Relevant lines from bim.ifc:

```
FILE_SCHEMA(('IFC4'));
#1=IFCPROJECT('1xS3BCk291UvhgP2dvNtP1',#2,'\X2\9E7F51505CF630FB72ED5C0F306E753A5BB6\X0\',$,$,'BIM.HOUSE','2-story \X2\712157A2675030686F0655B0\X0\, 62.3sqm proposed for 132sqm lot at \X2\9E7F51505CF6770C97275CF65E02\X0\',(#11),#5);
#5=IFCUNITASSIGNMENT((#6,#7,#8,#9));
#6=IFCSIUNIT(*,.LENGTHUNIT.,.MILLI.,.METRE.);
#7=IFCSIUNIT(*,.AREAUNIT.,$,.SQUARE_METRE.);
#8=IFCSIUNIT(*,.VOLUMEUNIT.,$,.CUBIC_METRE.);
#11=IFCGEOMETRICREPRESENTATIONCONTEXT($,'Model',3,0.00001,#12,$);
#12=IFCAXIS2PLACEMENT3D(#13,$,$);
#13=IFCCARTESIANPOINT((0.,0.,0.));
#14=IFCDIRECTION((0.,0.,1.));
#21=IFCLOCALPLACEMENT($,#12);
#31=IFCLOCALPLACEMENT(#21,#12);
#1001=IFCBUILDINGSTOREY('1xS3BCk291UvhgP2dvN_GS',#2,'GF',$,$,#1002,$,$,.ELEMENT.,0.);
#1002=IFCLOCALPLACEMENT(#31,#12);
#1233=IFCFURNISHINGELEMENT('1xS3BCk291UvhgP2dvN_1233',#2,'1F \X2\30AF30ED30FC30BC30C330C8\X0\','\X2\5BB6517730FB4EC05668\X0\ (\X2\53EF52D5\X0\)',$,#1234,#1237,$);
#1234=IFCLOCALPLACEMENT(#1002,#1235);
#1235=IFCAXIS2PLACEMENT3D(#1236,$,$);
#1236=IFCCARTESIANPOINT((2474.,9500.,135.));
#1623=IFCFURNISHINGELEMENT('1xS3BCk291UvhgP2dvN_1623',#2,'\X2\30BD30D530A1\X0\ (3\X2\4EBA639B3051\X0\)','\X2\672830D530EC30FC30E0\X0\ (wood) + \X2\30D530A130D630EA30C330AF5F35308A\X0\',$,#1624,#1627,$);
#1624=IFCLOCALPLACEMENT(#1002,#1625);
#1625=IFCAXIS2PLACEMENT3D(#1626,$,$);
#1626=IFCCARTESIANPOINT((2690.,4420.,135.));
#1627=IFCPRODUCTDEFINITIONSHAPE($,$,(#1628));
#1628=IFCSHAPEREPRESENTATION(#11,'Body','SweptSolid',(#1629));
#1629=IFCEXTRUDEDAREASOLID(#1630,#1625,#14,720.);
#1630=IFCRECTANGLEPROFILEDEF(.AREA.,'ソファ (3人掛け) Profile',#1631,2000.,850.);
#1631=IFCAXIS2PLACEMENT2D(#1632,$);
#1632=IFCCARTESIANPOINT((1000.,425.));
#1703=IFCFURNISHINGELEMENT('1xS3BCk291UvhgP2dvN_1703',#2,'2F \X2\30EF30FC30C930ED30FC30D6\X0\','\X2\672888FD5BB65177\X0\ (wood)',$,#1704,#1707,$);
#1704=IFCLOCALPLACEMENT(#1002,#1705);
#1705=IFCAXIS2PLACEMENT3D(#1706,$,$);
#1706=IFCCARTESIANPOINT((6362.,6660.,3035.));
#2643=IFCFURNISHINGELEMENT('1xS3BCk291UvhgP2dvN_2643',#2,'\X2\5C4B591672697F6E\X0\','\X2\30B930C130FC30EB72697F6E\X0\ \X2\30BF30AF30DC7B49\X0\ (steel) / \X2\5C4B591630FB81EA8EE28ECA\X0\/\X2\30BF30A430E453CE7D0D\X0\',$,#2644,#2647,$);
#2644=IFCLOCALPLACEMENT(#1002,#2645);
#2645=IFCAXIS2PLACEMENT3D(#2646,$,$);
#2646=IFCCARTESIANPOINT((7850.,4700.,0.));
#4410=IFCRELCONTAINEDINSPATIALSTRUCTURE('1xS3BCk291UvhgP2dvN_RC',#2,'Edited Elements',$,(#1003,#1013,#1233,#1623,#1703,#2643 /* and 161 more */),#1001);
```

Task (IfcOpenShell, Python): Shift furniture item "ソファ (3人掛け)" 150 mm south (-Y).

```python
import ifcopenshell
import ifcopenshell.api.geometry
import ifcopenshell.util.placement

model = ifcopenshell.open("bim.ifc")

item = model.by_guid("1xS3BCk291UvhgP2dvN_1623")
matrix = ifcopenshell.util.placement.get_local_placement(item.ObjectPlacement)
matrix[1, 3] -= 150.0
ifcopenshell.api.geometry.edit_object_placement(model, product=item, matrix=matrix, is_si=False)

print(ifcopenshell.util.placement.get_local_placement(item.ObjectPlacement).round(3) + 0.0)

model.write("bim-out.ifc")
```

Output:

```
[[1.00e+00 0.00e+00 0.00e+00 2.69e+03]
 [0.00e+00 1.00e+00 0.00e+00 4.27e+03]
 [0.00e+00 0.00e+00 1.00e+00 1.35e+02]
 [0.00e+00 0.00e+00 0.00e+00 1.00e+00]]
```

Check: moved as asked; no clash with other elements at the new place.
